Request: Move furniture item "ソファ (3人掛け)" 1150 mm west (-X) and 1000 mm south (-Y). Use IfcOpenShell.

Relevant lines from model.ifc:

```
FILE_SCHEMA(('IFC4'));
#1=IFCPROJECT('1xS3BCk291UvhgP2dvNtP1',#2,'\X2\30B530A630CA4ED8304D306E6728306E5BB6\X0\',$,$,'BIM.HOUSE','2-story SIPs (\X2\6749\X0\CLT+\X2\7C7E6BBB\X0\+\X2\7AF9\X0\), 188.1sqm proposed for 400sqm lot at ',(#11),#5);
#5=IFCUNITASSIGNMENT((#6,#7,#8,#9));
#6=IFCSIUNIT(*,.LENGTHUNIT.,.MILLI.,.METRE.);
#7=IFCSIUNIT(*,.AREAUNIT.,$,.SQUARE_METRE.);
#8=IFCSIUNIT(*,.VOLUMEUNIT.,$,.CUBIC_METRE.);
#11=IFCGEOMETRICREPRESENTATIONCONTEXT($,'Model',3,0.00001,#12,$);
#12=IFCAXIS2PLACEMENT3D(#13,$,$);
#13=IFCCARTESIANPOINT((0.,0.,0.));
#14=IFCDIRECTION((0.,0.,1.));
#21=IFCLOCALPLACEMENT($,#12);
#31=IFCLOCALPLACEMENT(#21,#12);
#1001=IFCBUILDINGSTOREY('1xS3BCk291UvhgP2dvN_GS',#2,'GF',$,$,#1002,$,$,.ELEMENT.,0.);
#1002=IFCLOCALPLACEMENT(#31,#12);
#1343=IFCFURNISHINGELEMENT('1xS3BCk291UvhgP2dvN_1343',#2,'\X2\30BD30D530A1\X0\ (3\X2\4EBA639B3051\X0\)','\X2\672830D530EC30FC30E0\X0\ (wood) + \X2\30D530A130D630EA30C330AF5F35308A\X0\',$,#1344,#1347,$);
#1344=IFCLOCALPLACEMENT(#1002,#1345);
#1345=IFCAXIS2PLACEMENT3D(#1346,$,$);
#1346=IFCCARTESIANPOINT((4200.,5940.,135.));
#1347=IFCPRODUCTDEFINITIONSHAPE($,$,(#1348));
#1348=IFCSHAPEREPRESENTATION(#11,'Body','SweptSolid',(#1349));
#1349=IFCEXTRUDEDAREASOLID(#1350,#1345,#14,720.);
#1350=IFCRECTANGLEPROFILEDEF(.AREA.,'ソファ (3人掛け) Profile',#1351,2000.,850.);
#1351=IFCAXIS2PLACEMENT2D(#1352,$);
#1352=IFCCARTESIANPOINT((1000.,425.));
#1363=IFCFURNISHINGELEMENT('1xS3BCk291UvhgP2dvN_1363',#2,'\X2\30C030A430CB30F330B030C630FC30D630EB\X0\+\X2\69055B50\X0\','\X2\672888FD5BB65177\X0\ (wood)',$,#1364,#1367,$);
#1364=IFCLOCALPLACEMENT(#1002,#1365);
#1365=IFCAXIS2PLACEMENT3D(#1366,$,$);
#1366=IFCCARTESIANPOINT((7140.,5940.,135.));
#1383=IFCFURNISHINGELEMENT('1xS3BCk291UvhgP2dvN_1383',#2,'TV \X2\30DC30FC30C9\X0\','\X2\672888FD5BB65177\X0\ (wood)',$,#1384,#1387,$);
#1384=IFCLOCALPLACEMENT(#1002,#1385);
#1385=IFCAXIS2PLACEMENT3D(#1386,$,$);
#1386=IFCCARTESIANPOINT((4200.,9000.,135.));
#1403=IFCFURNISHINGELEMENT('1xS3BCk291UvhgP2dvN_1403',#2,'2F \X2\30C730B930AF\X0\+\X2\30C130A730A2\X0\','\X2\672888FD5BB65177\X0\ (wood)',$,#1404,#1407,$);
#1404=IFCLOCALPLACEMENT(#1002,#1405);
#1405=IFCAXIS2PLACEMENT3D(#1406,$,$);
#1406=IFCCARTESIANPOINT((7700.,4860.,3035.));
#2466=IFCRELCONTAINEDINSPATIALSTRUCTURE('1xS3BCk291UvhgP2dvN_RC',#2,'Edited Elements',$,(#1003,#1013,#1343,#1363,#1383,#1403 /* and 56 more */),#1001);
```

```python
import ifcopenshell
import ifcopenshell.api.geometry
import ifcopenshell.util.placement

model = ifcopenshell.open("model.ifc")

item = model.by_guid("1xS3BCk291UvhgP2dvN_1343")
matrix = ifcopenshell.util.placement.get_local_placement(item.ObjectPlacement)
matrix[0, 3] -= 1150.0
matrix[1, 3] -= 1000.0
ifcopenshell.api.geometry.edit_object_placement(model, product=item, matrix=matrix, is_si=False)

print(ifcopenshell.util.placement.get_local_placement(item.ObjectPlacement).round(3) + 0.0)

model.write("model-out.ifc")
```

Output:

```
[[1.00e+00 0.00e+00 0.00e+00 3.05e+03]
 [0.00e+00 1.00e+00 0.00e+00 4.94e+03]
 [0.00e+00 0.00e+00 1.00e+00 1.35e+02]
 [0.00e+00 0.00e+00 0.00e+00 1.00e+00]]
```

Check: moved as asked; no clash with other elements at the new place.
